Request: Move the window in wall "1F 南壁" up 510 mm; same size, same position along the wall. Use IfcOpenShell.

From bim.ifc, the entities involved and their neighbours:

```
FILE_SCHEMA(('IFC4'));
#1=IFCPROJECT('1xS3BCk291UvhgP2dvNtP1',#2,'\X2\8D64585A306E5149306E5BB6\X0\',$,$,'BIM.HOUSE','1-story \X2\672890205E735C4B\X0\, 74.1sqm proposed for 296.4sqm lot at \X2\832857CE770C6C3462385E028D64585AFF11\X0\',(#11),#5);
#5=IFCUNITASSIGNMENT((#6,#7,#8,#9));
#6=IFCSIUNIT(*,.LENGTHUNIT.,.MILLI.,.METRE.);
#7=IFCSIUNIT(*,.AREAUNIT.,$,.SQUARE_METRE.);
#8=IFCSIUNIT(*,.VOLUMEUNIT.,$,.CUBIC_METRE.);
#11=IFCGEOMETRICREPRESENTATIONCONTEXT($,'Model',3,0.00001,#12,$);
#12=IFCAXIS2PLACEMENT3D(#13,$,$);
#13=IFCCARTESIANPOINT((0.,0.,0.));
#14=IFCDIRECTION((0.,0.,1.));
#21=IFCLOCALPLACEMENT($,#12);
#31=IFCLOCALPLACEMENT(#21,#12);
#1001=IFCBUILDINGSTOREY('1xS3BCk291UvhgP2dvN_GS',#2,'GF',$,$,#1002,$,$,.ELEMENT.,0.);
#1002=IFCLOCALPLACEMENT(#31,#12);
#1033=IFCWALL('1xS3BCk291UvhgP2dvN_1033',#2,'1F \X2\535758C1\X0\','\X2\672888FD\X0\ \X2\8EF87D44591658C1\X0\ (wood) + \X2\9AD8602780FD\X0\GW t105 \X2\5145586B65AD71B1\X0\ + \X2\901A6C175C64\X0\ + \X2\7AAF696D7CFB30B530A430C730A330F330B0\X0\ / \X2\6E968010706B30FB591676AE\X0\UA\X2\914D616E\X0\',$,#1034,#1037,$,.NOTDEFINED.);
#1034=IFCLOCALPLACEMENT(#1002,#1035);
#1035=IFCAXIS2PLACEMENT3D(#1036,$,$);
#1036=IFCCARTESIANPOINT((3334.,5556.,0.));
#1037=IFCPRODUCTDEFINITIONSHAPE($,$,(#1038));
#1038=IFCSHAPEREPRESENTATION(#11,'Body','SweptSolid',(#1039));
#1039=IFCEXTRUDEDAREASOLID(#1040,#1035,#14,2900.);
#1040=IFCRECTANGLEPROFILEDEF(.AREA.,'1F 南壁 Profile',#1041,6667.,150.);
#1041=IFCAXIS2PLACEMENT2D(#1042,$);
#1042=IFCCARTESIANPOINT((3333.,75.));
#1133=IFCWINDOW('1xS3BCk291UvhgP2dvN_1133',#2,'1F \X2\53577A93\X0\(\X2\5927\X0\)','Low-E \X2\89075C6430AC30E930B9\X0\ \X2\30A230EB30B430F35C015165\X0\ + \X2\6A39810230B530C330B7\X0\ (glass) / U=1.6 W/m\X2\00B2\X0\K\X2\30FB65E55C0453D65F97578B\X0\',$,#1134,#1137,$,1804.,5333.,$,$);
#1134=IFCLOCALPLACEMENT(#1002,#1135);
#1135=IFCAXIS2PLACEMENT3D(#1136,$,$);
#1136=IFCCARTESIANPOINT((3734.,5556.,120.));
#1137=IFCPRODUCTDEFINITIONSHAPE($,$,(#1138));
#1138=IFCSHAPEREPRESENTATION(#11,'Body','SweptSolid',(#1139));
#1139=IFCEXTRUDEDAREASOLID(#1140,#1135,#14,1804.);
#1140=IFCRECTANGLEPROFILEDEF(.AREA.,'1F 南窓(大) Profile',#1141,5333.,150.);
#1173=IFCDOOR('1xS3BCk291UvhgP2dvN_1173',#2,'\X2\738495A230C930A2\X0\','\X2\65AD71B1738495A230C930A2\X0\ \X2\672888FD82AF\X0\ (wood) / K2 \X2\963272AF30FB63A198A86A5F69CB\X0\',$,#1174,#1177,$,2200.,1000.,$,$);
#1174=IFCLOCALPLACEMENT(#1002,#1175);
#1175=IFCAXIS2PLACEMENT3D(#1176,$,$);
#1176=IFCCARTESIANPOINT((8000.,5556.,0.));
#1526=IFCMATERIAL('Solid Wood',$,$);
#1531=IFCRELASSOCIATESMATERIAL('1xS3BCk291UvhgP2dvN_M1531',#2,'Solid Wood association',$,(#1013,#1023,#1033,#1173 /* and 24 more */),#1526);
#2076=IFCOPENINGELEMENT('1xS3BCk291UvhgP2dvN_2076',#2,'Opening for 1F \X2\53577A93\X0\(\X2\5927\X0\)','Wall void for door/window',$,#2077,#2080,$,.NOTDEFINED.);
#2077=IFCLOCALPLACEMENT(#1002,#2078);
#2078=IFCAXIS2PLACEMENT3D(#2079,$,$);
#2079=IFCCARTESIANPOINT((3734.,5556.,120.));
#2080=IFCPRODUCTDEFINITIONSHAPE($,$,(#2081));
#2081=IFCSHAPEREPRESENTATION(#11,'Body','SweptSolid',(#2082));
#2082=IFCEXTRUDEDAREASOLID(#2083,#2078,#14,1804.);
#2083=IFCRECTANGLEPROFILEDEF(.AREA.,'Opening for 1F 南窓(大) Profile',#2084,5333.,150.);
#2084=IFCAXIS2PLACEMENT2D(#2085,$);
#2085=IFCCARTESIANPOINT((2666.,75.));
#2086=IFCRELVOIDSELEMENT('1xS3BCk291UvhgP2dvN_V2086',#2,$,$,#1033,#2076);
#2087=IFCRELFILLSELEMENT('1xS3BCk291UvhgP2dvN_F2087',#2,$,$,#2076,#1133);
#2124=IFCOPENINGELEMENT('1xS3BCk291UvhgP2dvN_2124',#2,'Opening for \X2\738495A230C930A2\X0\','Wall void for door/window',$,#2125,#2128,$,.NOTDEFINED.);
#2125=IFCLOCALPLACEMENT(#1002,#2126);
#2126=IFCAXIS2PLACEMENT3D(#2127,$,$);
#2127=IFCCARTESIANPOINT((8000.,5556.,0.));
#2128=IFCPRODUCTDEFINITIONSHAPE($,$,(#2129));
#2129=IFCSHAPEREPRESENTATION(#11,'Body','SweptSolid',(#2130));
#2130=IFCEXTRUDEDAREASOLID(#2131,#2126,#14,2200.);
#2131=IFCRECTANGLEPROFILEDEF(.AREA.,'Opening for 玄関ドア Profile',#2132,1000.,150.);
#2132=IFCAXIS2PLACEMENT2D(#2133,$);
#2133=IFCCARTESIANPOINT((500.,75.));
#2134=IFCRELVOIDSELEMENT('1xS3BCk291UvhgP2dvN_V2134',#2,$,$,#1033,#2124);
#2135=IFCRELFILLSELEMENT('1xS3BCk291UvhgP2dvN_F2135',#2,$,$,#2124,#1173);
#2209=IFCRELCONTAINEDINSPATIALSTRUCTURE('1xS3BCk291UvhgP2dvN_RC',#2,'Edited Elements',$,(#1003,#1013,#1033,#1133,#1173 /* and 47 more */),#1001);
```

```python
import numpy as np
import ifcopenshell
import ifcopenshell.api.geometry
import ifcopenshell.util.placement
import ifcopenshell.util.unit

model = ifcopenshell.open("bim.ifc")
unit_scale = ifcopenshell.util.unit.calculate_unit_scale(model)

window = model.by_id(1133)
opening = window.FillsVoids[0].RelatingOpeningElement
dz = 0.51 / unit_scale

shift = np.array([0.0, 0.0, dz])
# The window is not placed relative to its opening, so move both.
for product in (opening, window):
    matrix = ifcopenshell.util.placement.get_local_placement(product.ObjectPlacement)
    matrix[:3, 3] += shift
    ifcopenshell.api.geometry.edit_object_placement(model, product=product, matrix=matrix, is_si=False)

print(f"moved by {dz * unit_scale:+.3f} m")

model.write("bim_edited.ifc")
```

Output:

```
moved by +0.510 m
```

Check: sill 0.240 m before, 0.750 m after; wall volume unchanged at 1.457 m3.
